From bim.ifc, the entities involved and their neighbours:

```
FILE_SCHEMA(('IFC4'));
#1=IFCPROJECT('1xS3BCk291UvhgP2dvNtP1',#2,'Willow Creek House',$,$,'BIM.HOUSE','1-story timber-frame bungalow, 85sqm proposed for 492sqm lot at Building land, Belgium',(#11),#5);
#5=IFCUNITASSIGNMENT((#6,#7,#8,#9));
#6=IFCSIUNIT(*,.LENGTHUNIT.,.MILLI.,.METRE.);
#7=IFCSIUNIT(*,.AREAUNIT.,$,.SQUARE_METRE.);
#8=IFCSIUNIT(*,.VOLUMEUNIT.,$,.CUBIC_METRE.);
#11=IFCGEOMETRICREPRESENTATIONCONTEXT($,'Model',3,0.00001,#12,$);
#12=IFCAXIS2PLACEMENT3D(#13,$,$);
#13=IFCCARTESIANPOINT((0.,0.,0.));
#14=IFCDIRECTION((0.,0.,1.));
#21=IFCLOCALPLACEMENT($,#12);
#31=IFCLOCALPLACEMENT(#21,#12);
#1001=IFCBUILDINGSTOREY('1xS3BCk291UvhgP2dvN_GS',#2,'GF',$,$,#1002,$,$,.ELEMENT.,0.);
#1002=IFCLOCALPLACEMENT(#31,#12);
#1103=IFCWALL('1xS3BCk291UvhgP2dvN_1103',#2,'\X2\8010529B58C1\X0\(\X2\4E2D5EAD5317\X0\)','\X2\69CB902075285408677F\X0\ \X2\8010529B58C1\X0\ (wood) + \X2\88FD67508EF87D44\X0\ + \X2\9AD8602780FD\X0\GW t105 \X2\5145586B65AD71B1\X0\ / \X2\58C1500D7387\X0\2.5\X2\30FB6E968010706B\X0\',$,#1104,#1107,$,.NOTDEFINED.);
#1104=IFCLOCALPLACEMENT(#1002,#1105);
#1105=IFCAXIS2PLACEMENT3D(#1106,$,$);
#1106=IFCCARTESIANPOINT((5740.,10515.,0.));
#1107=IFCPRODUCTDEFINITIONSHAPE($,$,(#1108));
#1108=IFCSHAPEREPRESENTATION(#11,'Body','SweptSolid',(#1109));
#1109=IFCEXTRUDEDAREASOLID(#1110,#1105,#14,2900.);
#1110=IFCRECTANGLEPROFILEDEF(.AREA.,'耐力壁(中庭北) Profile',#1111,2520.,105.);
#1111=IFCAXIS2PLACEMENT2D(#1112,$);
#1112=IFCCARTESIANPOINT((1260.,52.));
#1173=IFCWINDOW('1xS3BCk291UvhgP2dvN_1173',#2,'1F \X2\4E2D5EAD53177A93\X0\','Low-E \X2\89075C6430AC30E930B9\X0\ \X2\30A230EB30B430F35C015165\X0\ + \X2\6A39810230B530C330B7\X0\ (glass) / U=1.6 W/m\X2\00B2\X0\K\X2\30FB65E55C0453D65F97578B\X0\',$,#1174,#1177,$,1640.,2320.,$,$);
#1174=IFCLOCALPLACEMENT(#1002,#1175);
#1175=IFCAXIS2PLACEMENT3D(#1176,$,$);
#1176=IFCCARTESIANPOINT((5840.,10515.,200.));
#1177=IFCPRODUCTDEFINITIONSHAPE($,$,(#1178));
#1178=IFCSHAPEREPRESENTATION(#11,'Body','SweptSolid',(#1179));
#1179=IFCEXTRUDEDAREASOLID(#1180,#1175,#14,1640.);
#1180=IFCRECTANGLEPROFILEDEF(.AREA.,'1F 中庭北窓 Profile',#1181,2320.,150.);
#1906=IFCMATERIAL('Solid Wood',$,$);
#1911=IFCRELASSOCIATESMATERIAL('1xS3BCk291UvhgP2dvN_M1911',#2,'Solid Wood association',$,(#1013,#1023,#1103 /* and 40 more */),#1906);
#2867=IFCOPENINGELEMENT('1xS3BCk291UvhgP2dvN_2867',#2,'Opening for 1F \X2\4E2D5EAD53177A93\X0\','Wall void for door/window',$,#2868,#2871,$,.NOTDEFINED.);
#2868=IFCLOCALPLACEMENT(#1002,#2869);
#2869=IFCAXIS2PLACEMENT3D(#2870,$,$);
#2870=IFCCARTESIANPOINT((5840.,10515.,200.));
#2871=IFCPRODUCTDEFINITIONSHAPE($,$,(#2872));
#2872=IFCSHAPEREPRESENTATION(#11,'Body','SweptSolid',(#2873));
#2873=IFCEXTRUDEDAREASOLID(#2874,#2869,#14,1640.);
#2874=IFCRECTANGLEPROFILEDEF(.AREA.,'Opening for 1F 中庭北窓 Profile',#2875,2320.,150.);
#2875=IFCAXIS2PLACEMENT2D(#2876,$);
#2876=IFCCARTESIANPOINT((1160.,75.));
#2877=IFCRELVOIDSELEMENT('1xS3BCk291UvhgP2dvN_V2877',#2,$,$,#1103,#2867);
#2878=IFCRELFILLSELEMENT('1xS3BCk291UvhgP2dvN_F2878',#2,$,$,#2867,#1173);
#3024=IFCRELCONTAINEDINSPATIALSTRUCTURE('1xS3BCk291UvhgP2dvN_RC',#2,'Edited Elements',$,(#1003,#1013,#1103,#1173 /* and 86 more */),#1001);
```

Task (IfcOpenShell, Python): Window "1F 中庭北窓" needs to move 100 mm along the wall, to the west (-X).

```python
import ifcopenshell
import ifcopenshell.api.geometry
import ifcopenshell.util.placement

model = ifcopenshell.open("bim.ifc")

window = model.by_guid("1xS3BCk291UvhgP2dvN_1173")
opening = window.FillsVoids[0].RelatingOpeningElement
wall = opening.VoidsElements[0].RelatingBuildingElement

wall_matrix = ifcopenshell.util.placement.get_local_placement(wall.ObjectPlacement)
shift = wall_matrix[:3, 0] * -100.0
before = ifcopenshell.util.placement.get_local_placement(window.ObjectPlacement)[:3, 3].copy()

# The window is not placed relative to its opening, so move both.
for product in (opening, window):
    matrix = ifcopenshell.util.placement.get_local_placement(product.ObjectPlacement)
    matrix[:3, 3] += shift
    ifcopenshell.api.geometry.edit_object_placement(model, product=product, matrix=matrix, is_si=False)

after = ifcopenshell.util.placement.get_local_placement(window.ObjectPlacement)[:3, 3]
print("window moved by", (after - before).round(3) + 0.0)

model.write("bim_updated.ifc")
```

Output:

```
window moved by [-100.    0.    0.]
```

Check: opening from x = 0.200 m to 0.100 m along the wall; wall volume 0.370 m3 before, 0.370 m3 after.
